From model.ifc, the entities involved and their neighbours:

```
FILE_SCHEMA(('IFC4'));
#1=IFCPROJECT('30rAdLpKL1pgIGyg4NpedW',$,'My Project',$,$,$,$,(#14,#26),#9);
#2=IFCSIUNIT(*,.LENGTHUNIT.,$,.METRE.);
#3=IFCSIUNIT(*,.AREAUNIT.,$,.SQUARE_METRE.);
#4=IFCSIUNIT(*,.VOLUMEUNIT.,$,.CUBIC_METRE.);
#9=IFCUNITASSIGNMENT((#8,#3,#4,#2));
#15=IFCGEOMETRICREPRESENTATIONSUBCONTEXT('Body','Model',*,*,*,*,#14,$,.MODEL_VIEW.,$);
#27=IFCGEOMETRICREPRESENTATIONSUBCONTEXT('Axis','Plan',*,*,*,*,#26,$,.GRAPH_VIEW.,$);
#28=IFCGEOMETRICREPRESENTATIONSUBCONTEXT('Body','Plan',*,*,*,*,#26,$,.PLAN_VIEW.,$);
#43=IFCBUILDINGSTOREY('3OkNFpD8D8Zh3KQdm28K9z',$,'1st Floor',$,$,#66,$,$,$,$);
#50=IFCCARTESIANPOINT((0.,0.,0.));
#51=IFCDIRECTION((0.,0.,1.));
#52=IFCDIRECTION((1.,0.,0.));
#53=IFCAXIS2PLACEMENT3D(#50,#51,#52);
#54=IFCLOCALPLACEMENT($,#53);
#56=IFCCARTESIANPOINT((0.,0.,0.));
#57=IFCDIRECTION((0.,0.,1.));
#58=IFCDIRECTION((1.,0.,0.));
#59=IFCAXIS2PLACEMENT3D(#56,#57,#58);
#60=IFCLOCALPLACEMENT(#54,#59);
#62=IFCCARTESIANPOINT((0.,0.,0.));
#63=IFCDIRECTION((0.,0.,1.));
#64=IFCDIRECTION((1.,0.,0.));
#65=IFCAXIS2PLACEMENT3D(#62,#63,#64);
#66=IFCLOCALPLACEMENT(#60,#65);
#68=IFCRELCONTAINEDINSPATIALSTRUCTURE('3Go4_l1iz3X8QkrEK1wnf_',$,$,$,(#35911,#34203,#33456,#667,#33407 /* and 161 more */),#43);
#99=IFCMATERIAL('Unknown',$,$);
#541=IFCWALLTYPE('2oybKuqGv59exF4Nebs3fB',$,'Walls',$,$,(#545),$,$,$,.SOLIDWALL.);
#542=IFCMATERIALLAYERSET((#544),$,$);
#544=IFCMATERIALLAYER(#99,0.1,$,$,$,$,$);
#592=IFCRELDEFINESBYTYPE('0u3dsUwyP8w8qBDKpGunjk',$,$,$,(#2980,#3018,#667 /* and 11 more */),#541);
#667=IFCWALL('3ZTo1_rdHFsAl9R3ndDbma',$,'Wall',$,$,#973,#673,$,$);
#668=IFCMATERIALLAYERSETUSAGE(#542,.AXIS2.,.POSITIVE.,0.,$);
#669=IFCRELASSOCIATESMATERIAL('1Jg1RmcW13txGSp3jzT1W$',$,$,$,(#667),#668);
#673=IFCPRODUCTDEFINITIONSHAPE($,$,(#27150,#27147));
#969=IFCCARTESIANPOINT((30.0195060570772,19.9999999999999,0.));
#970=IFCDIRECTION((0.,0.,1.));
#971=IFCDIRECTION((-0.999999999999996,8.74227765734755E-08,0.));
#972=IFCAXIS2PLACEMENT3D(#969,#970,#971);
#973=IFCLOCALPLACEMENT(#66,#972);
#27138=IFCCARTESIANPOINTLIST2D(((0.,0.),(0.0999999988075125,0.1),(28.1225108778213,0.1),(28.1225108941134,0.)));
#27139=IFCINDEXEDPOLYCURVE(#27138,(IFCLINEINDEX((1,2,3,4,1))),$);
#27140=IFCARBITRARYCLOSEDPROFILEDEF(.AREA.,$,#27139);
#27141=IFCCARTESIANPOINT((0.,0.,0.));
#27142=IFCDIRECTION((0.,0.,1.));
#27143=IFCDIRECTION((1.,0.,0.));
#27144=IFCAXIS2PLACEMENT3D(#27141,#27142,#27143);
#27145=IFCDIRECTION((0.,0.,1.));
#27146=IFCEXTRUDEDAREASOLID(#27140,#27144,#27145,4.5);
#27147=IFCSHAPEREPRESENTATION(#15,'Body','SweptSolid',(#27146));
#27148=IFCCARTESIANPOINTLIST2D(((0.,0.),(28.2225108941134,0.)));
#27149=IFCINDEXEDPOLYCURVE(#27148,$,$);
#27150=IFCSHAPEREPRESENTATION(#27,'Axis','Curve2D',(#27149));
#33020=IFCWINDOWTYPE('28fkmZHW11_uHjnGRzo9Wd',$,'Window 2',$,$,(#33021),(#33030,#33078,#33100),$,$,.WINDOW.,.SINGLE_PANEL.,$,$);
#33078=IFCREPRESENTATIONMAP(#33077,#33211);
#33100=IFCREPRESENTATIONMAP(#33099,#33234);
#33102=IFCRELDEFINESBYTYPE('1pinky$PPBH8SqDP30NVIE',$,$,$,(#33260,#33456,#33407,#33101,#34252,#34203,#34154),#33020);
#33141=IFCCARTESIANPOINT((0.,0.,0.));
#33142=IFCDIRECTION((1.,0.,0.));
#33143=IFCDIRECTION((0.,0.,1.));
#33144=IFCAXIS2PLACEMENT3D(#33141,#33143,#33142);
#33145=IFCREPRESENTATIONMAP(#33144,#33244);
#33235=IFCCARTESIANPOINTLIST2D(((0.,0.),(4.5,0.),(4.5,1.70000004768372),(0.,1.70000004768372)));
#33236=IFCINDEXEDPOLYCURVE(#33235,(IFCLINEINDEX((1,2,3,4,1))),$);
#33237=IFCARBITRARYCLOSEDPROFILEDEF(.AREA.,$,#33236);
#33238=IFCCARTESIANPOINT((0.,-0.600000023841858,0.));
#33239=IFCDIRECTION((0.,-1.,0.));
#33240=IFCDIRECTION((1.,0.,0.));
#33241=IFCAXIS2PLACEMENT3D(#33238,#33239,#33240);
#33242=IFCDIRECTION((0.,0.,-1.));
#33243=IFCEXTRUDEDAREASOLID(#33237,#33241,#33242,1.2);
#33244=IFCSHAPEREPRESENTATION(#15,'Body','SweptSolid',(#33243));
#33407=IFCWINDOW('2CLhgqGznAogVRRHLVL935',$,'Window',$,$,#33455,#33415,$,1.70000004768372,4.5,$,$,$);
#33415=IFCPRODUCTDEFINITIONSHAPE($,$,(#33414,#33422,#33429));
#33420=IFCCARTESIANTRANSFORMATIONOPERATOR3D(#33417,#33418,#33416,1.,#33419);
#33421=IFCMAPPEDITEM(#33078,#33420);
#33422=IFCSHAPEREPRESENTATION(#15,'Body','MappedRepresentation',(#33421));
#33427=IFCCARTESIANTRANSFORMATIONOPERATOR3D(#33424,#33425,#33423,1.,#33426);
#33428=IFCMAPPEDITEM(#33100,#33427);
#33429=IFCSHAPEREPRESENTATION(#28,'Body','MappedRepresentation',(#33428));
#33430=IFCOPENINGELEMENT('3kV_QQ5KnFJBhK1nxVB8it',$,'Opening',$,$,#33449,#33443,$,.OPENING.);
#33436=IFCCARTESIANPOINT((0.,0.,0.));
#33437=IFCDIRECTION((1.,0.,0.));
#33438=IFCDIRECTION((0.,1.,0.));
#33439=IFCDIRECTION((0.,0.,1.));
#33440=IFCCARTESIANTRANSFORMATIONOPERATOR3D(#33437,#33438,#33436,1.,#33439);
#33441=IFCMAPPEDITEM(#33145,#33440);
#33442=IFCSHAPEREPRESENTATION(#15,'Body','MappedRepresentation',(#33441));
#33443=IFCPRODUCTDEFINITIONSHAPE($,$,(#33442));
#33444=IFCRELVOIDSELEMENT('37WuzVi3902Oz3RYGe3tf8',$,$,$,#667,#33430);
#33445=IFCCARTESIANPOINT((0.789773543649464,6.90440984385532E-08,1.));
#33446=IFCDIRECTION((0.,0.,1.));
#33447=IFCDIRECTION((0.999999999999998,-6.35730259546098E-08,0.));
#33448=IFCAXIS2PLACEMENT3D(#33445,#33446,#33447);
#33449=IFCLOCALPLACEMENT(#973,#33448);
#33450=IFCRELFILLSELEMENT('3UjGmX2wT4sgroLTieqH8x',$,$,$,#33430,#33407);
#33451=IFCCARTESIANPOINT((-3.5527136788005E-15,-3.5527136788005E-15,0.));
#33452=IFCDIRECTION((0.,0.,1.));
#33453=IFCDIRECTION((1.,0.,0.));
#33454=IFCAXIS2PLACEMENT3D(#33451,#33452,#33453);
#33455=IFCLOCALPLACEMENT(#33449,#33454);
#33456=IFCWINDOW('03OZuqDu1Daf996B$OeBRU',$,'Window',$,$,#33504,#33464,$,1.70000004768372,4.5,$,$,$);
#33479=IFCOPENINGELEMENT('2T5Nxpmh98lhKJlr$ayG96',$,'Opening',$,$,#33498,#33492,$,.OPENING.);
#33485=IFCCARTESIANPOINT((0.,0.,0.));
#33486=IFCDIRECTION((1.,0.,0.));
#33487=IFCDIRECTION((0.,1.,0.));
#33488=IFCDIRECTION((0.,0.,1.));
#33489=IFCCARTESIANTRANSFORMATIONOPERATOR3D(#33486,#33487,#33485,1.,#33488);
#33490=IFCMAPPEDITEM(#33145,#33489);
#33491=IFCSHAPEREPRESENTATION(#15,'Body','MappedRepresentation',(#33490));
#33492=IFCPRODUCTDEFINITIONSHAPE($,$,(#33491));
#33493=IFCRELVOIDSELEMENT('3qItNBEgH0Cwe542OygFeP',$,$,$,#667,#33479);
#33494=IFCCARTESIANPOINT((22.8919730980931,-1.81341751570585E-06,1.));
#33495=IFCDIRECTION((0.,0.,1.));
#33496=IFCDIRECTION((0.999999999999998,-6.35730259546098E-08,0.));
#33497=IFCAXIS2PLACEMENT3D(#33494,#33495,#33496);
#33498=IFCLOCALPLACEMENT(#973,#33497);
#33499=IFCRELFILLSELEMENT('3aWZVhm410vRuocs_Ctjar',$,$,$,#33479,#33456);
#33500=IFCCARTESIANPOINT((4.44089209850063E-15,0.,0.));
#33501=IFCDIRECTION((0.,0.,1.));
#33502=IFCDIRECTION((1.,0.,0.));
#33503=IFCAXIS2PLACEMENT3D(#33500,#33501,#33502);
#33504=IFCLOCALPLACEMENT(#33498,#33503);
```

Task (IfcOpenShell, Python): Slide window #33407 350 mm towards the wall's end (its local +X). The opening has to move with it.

```python
import ifcopenshell
import ifcopenshell.api.geometry
import ifcopenshell.util.placement
import ifcopenshell.util.unit

model = ifcopenshell.open("model.ifc")
unit_scale = ifcopenshell.util.unit.calculate_unit_scale(model)

window = model.by_guid("2CLhgqGznAogVRRHLVL935")
opening = window.FillsVoids[0].RelatingOpeningElement
wall = opening.VoidsElements[0].RelatingBuildingElement

wall_matrix = ifcopenshell.util.placement.get_local_placement(wall.ObjectPlacement)
shift = wall_matrix[:3, 0] * 0.35 / unit_scale
before = ifcopenshell.util.placement.get_local_placement(window.ObjectPlacement)[:3, 3].copy()

# The window is placed relative to its opening, so it follows when the opening moves.
matrix = ifcopenshell.util.placement.get_local_placement(opening.ObjectPlacement)
matrix[:3, 3] += shift
ifcopenshell.api.geometry.edit_object_placement(
    model, product=opening, matrix=matrix, is_si=False, should_transform_children=True
)

after = ifcopenshell.util.placement.get_local_placement(window.ObjectPlacement)[:3, 3]
print("window moved by", (after - before).round(3) + 0.0)

model.write("model-out.ifc")
```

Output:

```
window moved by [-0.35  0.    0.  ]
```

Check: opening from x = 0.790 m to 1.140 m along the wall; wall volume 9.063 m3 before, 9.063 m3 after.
